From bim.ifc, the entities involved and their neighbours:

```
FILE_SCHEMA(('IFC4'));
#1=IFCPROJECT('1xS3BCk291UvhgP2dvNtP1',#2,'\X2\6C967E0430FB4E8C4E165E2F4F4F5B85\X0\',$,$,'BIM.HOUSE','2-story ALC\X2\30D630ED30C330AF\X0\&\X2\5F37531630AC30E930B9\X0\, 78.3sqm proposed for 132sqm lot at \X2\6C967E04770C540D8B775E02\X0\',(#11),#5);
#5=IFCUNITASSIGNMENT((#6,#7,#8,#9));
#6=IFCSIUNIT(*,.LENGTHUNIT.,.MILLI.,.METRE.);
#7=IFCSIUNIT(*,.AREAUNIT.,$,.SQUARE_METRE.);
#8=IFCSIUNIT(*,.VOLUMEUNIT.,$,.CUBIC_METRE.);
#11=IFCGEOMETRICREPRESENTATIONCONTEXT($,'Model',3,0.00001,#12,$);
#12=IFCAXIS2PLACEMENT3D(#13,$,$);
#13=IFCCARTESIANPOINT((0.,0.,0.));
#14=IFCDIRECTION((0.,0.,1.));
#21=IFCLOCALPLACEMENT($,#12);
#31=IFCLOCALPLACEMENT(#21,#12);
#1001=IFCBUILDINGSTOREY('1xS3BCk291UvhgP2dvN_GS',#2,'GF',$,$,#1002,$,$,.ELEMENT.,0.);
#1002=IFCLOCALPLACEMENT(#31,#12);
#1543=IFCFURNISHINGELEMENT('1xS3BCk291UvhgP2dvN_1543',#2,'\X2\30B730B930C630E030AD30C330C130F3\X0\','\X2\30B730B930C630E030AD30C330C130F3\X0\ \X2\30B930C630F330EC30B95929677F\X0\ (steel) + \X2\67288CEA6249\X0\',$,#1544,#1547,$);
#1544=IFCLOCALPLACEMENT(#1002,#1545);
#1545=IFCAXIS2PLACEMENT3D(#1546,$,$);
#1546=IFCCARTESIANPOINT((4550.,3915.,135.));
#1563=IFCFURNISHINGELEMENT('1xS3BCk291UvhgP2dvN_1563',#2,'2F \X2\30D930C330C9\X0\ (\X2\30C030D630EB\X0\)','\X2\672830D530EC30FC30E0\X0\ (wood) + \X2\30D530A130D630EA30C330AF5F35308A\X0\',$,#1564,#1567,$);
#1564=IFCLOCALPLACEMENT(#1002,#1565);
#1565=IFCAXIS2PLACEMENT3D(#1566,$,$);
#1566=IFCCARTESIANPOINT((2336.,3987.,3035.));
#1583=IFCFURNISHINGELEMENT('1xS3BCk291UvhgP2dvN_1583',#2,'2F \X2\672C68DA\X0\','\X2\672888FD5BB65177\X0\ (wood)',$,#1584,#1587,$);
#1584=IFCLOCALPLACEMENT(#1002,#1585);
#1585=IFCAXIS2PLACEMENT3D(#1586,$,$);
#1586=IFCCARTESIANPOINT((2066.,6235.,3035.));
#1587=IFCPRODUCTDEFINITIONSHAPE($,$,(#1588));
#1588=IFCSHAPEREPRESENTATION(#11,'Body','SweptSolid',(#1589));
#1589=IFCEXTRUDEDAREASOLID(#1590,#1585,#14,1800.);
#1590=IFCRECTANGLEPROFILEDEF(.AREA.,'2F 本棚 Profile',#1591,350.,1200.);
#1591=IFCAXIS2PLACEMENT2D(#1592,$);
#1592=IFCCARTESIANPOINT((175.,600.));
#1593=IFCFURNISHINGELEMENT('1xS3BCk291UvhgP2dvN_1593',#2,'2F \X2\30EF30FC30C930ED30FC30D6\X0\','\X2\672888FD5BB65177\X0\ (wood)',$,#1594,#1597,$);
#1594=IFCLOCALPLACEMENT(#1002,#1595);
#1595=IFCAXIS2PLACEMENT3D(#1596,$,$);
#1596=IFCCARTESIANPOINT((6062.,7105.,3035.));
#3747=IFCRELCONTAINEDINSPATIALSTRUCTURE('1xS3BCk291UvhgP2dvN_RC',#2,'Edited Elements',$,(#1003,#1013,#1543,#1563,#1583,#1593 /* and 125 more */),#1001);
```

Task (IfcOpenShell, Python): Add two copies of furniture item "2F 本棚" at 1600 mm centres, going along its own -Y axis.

```python
import ifcopenshell
import ifcopenshell.api.geometry
import ifcopenshell.api.root
import ifcopenshell.util.element
import ifcopenshell.util.placement

model = ifcopenshell.open("bim.ifc")


def reuse_history(source, copy):
    """copy_class also copies each property set's owner history, people and application; keep the originals."""
    for rel in copy.IsDefinedBy:
        if rel.is_a("IfcRelDefinesByProperties") and (history := rel.RelatingPropertyDefinition.OwnerHistory):
            rel.RelatingPropertyDefinition.OwnerHistory = source.OwnerHistory
            ifcopenshell.util.element.remove_deep2(model, history)


source = model.by_guid("1xS3BCk291UvhgP2dvN_1583")
base = ifcopenshell.util.placement.get_local_placement(source.ObjectPlacement)
step = -base[:3, 1] * 1600.0

for i in range(1, 3):
    copy = ifcopenshell.api.root.copy_class(model, product=source)
    copy.Representation = ifcopenshell.util.element.copy_deep(
        model, source.Representation, exclude=["IfcGeometricRepresentationContext", "IfcRepresentationMap"]
    )
    reuse_history(source, copy)
    matrix = base.copy()
    matrix[:3, 3] += i * step
    print("added at", matrix[:3, 3].round(3) + 0.0)
    ifcopenshell.api.geometry.edit_object_placement(model, product=copy, matrix=matrix, is_si=False)

model.write("bim-out.ifc")
```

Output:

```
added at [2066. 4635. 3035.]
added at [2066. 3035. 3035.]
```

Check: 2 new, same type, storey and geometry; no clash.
